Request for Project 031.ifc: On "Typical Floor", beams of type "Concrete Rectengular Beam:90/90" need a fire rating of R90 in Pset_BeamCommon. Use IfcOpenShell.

First a look at what the model holds.

```python
import ifcopenshell
import ifcopenshell.util.element

model = ifcopenshell.open("Project 031.ifc")
print(model.schema)
storey = next(s for s in model.by_type("IfcBuildingStorey") if s.Name == "Typical Floor")
beams = [e for e in ifcopenshell.util.element.get_decomposition(storey) if e.is_a("IfcBeam")]
seen = {}
for e in beams:
    element_type = ifcopenshell.util.element.get_type(e)
    key = (element_type.Name if element_type != e and element_type else None, ifcopenshell.util.element.get_pset(e, "Pset_BeamCommon", "FireRating"))
    seen[key] = seen.get(key, 0) + 1
for (name, value), count in sorted(seen.items(), key=str):
    print(count, "x", name, "|", value)
```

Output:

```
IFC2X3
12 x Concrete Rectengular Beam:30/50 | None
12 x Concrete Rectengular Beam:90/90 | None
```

```python
import ifcopenshell
import ifcopenshell.api.pset
import ifcopenshell.util.element

model = ifcopenshell.open("Project 031.ifc")

storey = next(s for s in model.by_type("IfcBuildingStorey") if s.Name == "Typical Floor")
beams = [e for e in ifcopenshell.util.element.get_decomposition(storey) if e.is_a("IfcBeam")]

count = 0
for e in beams:
    element_type = ifcopenshell.util.element.get_type(e)
    if element_type in (None, e) or element_type.Name != "Concrete Rectengular Beam:90/90":
        continue
    # add_pset returns the element's existing set when there is one.
    pset = ifcopenshell.api.pset.add_pset(model, product=e, name="Pset_BeamCommon")
    ifcopenshell.api.pset.edit_pset(model, pset=pset, properties={"FireRating": "R90"})
    count += 1

print(count, "beams updated")

model.write("Project 031-out.ifc")
```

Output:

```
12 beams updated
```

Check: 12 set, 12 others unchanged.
